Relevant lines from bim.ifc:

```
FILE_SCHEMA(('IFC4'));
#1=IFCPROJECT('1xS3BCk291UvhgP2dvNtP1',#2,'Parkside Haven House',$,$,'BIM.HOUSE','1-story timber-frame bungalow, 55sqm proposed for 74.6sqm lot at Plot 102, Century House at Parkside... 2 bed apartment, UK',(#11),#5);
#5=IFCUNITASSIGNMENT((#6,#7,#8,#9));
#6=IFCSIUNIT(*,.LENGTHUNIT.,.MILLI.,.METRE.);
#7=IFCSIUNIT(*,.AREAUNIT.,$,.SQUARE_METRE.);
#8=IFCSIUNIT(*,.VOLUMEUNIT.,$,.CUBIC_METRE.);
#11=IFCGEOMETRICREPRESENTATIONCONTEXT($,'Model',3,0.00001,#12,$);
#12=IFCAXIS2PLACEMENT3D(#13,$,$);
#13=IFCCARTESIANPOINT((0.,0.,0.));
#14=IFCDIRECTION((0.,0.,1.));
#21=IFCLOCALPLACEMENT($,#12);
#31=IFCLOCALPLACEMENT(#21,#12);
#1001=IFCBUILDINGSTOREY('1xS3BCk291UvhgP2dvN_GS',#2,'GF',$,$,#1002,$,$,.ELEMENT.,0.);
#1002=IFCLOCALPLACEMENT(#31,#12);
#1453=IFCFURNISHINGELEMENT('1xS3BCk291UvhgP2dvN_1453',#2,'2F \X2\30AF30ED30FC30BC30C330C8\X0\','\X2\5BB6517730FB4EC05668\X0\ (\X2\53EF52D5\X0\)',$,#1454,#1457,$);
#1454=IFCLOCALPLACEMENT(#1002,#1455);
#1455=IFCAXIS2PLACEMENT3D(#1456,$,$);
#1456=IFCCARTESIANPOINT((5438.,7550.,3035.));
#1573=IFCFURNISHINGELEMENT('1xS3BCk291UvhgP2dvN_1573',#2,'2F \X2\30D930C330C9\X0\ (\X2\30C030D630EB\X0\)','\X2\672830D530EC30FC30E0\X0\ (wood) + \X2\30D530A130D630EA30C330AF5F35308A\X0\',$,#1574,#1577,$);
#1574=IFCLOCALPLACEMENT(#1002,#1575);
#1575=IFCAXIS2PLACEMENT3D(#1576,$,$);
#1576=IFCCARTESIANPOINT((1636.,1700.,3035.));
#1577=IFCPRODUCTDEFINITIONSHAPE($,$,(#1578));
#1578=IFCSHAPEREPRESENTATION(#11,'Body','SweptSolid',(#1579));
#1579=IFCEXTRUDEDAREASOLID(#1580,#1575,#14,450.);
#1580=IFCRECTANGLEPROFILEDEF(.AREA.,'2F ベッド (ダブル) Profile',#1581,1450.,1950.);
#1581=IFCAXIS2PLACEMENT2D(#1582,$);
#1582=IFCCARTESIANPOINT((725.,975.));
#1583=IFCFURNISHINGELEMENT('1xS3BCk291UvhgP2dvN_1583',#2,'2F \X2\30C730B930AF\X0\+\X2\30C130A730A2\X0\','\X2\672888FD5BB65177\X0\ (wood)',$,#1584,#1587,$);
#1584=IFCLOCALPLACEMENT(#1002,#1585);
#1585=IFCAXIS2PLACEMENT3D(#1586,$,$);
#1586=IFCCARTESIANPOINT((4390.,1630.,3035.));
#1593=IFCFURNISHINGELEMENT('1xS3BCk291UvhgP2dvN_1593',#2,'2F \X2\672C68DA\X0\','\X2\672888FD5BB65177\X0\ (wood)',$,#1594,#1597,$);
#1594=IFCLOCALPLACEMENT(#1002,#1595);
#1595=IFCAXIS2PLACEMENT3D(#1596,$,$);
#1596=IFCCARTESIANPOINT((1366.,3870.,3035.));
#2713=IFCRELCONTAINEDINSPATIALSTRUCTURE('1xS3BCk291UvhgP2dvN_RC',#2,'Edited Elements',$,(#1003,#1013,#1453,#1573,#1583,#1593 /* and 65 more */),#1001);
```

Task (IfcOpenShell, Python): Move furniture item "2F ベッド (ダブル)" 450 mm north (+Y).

```python
import ifcopenshell
import ifcopenshell.api.geometry
import ifcopenshell.util.placement

model = ifcopenshell.open("bim.ifc")

item = model.by_guid("1xS3BCk291UvhgP2dvN_1573")
matrix = ifcopenshell.util.placement.get_local_placement(item.ObjectPlacement)
matrix[1, 3] += 450.0
ifcopenshell.api.geometry.edit_object_placement(model, product=item, matrix=matrix, is_si=False)

print(ifcopenshell.util.placement.get_local_placement(item.ObjectPlacement).round(3) + 0.0)

model.write("bim_rev.ifc")
```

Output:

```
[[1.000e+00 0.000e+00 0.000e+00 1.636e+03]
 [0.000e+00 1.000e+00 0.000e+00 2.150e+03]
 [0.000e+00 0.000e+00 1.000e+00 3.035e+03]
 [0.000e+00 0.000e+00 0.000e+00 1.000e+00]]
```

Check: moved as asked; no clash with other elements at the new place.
